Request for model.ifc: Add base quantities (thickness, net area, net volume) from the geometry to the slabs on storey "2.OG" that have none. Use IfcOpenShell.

First a look at what the model holds.

```python
import ifcopenshell
import ifcopenshell.util.element
import ifcopenshell.util.unit

model = ifcopenshell.open("model.ifc")
print(model.schema)
for unit_type in ("LENGTHUNIT", "AREAUNIT", "VOLUMEUNIT"):
    print(unit_type, ifcopenshell.util.unit.calculate_unit_scale(model, unit_type))
storey = next(s for s in model.by_type("IfcBuildingStorey") if s.Name == "2.OG")
slabs = [e for e in ifcopenshell.util.element.get_decomposition(storey) if e.is_a("IfcSlab")]
for e in sorted(slabs, key=lambda e: e.id()):
    print(e.id(), e.is_a(), e.Name, list(ifcopenshell.util.element.get_psets(e, qtos_only=True)), sep=" | ")
```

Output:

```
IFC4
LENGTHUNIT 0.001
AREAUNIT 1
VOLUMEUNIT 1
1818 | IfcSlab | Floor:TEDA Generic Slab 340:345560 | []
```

```python
import ifcopenshell
import ifcopenshell.api.pset
import ifcopenshell.geom
import ifcopenshell.util.element
import ifcopenshell.util.shape
import ifcopenshell.util.unit

model = ifcopenshell.open("model.ifc")
unit_scale = ifcopenshell.util.unit.calculate_unit_scale(model)
area_scale = ifcopenshell.util.unit.calculate_unit_scale(model, "AREAUNIT")
volume_scale = ifcopenshell.util.unit.calculate_unit_scale(model, "VOLUMEUNIT")
settings = ifcopenshell.geom.settings()

storey = next(s for s in model.by_type("IfcBuildingStorey") if s.Name == "2.OG")
slabs = [e for e in ifcopenshell.util.element.get_decomposition(storey) if e.is_a("IfcSlab")]

for e in sorted(slabs, key=lambda e: e.id()):
    if ifcopenshell.util.element.get_psets(e, qtos_only=True, should_inherit=False):
        continue
    # Geometry comes back in metres, in the element's own axes.
    shape = ifcopenshell.geom.create_shape(settings, e)
    values = {
        "Width": ifcopenshell.util.shape.get_z(shape.geometry) / unit_scale,
        "NetArea": ifcopenshell.util.shape.get_footprint_area(shape.geometry) / area_scale,
        "NetVolume": ifcopenshell.util.shape.get_volume(shape.geometry) / volume_scale,
    }
    qto = ifcopenshell.api.pset.add_qto(model, product=e, name="Qto_SlabBaseQuantities")
    ifcopenshell.api.pset.edit_qto(model, qto=qto, properties=values)
    print(e.id(), {k: round(v, 3) for k, v in values.items()})

model.write("model-out.ifc")
```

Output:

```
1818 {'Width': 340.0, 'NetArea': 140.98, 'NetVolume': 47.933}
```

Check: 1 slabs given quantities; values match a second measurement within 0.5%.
